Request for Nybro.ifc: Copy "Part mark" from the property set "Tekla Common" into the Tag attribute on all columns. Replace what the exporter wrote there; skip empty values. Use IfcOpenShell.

First a look at what the model holds.

```python
import ifcopenshell
import ifcopenshell.util.element

model = ifcopenshell.open("Nybro.ifc")
print(model.schema)
columns = model.by_type("IfcColumn")
print(len(columns), "columns")
for e in columns[:8]:
    source = ifcopenshell.util.element.get_pset(e, "Tekla Common", "Part mark")
    target = e.Tag
    print(e.id(), repr(source), repr(target), sep=" | ")
```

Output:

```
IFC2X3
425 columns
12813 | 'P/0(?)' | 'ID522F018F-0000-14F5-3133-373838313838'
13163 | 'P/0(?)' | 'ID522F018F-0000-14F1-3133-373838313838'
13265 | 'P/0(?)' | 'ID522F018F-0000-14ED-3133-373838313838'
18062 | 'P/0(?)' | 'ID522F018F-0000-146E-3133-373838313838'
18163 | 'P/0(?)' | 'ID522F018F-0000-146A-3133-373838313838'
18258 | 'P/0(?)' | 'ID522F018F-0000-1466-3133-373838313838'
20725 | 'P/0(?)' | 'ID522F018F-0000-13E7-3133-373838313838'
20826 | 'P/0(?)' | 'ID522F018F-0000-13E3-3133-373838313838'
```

```python
import ifcopenshell
import ifcopenshell.util.element

model = ifcopenshell.open("Nybro.ifc")

count = 0
for e in model.by_type("IfcColumn"):
    value = ifcopenshell.util.element.get_pset(e, "Tekla Common", "Part mark")
    current = e.Tag
    if not value or not value.strip() or current == value:
        continue
    e.Tag = value
    count += 1

print(count, "columns updated")

model.write("Nybro-out.ifc")
```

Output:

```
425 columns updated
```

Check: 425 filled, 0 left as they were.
